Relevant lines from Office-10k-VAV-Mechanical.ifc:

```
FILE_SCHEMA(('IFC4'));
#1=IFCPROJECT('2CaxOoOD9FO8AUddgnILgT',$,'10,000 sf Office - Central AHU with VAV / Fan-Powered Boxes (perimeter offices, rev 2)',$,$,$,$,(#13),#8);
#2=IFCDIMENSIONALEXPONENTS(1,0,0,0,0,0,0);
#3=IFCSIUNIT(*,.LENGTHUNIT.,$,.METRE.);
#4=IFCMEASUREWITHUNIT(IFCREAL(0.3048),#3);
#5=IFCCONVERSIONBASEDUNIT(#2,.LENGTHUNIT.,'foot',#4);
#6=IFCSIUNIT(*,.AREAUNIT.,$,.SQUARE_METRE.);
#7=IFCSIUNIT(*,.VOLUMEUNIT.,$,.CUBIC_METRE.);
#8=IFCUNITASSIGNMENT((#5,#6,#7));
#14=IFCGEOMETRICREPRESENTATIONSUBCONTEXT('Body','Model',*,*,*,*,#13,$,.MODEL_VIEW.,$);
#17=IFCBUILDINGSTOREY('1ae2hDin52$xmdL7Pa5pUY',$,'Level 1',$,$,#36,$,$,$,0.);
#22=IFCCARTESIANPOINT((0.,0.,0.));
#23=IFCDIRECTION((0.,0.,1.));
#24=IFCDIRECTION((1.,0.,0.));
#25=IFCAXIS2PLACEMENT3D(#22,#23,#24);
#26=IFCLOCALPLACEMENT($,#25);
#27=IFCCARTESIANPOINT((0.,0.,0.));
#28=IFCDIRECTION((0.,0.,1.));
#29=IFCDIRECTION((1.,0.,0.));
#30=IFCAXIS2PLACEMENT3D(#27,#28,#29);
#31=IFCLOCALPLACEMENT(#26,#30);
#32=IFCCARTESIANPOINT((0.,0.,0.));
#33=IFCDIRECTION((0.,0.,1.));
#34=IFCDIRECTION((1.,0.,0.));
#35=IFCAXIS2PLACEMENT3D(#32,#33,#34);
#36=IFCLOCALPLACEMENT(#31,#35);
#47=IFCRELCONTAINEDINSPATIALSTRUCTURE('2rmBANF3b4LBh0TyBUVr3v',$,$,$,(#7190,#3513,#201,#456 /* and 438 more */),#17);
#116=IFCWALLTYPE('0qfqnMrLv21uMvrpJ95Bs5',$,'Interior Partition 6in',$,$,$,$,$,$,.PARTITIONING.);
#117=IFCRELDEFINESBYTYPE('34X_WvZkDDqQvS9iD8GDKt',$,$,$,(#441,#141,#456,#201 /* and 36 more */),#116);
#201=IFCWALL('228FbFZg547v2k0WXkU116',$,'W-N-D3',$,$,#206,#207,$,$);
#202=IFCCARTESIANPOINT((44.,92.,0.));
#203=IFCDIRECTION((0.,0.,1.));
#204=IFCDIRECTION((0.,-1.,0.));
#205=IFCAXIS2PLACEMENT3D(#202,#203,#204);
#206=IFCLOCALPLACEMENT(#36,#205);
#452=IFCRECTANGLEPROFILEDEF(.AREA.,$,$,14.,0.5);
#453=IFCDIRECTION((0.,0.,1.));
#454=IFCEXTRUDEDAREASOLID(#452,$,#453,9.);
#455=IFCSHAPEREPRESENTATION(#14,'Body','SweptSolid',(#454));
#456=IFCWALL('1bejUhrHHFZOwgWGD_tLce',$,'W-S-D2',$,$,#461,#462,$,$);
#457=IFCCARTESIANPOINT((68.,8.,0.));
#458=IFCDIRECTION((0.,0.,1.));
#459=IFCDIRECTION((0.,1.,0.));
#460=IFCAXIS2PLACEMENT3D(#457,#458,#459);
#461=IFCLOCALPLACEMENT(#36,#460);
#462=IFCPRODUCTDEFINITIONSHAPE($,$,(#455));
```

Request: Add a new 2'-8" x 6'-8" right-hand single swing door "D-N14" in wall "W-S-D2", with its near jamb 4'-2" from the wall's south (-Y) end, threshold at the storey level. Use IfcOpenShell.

```python
import numpy as np
import ifcopenshell
import ifcopenshell.api.feature
import ifcopenshell.api.geometry
import ifcopenshell.api.root
import ifcopenshell.api.spatial
import ifcopenshell.geom
import ifcopenshell.util.element
import ifcopenshell.util.placement
import ifcopenshell.util.representation
import ifcopenshell.util.shape
import ifcopenshell.util.unit

model = ifcopenshell.open("Office-10k-VAV-Mechanical.ifc")
unit_scale = ifcopenshell.util.unit.calculate_unit_scale(model)
settings = ifcopenshell.geom.settings()


def volume(element):
    """Net volume in cubic metres, openings subtracted."""
    shape = ifcopenshell.geom.create_shape(settings, element)
    return ifcopenshell.util.shape.get_volume(shape.geometry)


wall = model.by_id(456)
storey = ifcopenshell.util.element.get_container(wall, ifc_class="IfcBuildingStorey")
context = ifcopenshell.util.representation.get_context(model, "Model", "Body", "MODEL_VIEW")
before = volume(wall)

width, height, from_end, sill = 0.8128, 2.032, 1.27, 0.0  # metres

# The wall runs along its own X axis, and the end named is its -X end.
wall_shape = ifcopenshell.geom.create_shape(settings, wall)
x, y, z = ifcopenshell.util.shape.get_vertices(wall_shape.geometry).T
start = x.min() + from_end
face, thickness = float(y.min()), float(y.max() - y.min())
wall_matrix = ifcopenshell.util.placement.get_local_placement(wall.ObjectPlacement)
level = ifcopenshell.util.placement.get_local_placement(storey.ObjectPlacement)[2, 3]


def in_wall(x, y):
    """Placement at x, y metres in the wall's axes, at sill height."""
    matrix = wall_matrix.copy()
    matrix[:, 3] = wall_matrix @ np.array([x / unit_scale, y / unit_scale, 0.0, 1.0])
    matrix[2, 3] = level + sill / unit_scale
    return matrix


# Opening: a box that overshoots both wall faces by 50 mm.
opening = ifcopenshell.api.root.create_entity(model, ifc_class="IfcOpeningElement", predefined_type="OPENING")
box = ifcopenshell.api.geometry.add_wall_representation(
    model, context=context, length=width, height=height, thickness=thickness + 0.1
)
ifcopenshell.api.geometry.assign_representation(model, product=opening, representation=box)
ifcopenshell.api.geometry.edit_object_placement(model, product=opening, matrix=in_wall(start, face - 0.05), is_si=False)
ifcopenshell.api.feature.add_feature(model, feature=opening, element=wall)

door = ifcopenshell.api.root.create_entity(model, ifc_class="IfcDoor", name="D-N14", predefined_type="DOOR")
door.OverallWidth, door.OverallHeight = width / unit_scale, height / unit_scale
door.OperationType = "SINGLE_SWING_RIGHT"
body = ifcopenshell.api.geometry.add_door_representation(
    model,
    context=context,
    overall_width=door.OverallWidth,
    overall_height=door.OverallHeight,
    operation_type="SINGLE_SWING_RIGHT",
    lining_properties={"LiningDepth": thickness / unit_scale, "ThresholdDepth": thickness / unit_scale},
)
ifcopenshell.api.geometry.assign_representation(model, product=door, representation=body)
ifcopenshell.api.spatial.assign_container(model, products=[door], relating_structure=storey)
ifcopenshell.api.feature.add_filling(model, opening=opening, element=door)

# The lining spans the wall, so the door starts at the wall face.
ifcopenshell.api.geometry.edit_object_placement(model, product=door, matrix=in_wall(start, face), is_si=False)

after = volume(wall)

print(f"wall volume {before:.3f} -> {after:.3f} m3")

model.write("Office-10k-VAV-Mechanical_edited.ifc")
```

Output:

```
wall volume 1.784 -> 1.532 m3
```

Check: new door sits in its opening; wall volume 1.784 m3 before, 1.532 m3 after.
